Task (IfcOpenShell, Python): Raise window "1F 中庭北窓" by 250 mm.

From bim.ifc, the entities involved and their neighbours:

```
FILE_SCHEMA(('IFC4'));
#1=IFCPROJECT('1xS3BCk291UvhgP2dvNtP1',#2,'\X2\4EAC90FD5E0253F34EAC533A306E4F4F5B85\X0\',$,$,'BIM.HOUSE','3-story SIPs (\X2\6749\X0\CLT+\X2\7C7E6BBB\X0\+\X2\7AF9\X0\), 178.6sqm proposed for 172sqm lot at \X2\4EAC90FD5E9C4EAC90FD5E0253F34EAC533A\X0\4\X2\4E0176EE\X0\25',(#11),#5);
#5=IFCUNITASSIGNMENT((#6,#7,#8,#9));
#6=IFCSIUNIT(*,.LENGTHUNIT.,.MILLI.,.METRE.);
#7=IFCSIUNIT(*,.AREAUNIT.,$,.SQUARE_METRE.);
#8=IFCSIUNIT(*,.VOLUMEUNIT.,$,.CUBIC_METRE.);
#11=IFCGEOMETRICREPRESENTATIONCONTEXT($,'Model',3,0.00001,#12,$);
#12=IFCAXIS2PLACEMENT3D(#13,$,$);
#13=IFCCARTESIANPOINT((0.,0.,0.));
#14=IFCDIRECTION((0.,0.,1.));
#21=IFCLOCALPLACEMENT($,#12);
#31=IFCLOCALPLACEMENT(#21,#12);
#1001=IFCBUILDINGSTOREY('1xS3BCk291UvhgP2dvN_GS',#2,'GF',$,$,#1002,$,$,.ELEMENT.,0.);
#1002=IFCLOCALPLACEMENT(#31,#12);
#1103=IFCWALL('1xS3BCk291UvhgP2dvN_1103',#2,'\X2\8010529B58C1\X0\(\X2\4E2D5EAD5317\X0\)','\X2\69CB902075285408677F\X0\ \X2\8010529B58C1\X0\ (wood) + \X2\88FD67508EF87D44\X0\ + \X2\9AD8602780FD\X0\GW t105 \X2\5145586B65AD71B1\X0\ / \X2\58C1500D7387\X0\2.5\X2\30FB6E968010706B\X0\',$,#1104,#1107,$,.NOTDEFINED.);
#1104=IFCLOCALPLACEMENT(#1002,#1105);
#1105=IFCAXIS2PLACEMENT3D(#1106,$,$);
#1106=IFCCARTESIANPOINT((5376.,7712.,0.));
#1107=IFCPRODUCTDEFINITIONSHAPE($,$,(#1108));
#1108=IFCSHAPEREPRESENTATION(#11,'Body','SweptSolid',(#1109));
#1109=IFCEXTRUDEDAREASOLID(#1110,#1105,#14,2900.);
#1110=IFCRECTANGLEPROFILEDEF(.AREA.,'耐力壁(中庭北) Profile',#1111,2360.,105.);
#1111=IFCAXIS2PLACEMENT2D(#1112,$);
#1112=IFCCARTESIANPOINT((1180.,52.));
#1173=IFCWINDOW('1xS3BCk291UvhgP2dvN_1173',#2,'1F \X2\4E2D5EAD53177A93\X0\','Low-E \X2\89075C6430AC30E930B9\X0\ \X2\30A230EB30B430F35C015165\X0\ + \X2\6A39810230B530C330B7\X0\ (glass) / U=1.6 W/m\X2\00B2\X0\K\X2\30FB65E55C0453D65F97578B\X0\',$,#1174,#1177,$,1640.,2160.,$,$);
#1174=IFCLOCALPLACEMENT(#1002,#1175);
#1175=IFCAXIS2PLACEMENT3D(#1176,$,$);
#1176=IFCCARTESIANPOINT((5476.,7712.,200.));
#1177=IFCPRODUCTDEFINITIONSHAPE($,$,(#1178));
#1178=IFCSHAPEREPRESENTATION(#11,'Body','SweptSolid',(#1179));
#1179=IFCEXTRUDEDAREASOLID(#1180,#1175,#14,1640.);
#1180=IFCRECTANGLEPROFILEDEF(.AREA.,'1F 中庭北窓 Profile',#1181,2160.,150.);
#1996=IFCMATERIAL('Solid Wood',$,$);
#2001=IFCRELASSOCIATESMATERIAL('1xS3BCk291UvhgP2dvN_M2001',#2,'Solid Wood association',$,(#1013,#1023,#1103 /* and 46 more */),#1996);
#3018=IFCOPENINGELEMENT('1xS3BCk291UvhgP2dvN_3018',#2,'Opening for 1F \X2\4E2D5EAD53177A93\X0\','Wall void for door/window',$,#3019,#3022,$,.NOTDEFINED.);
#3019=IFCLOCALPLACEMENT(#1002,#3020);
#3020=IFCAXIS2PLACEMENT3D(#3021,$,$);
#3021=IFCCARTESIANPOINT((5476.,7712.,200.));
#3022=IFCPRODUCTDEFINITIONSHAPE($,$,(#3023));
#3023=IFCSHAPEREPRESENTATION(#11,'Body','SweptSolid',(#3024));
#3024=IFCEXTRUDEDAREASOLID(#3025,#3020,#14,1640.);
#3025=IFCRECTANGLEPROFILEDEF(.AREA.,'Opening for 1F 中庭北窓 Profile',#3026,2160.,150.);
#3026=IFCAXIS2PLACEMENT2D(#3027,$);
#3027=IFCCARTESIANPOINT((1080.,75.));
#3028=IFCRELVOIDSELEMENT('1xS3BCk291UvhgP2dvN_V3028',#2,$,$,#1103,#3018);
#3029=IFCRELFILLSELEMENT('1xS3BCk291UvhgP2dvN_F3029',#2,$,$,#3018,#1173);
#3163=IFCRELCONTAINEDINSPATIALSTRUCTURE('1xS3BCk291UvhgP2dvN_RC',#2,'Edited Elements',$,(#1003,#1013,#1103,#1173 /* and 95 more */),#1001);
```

```python
import numpy as np
import ifcopenshell
import ifcopenshell.api.geometry
import ifcopenshell.util.placement
import ifcopenshell.util.unit

model = ifcopenshell.open("bim.ifc")
unit_scale = ifcopenshell.util.unit.calculate_unit_scale(model)

window = model.by_id(1173)
opening = window.FillsVoids[0].RelatingOpeningElement
dz = 0.25 / unit_scale

shift = np.array([0.0, 0.0, dz])
# The window is not placed relative to its opening, so move both.
for product in (opening, window):
    matrix = ifcopenshell.util.placement.get_local_placement(product.ObjectPlacement)
    matrix[:3, 3] += shift
    ifcopenshell.api.geometry.edit_object_placement(model, product=product, matrix=matrix, is_si=False)

print(f"moved by {dz * unit_scale:+.3f} m")

model.write("bim_rev.ifc")
```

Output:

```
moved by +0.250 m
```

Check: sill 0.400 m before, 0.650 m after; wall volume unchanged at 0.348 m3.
